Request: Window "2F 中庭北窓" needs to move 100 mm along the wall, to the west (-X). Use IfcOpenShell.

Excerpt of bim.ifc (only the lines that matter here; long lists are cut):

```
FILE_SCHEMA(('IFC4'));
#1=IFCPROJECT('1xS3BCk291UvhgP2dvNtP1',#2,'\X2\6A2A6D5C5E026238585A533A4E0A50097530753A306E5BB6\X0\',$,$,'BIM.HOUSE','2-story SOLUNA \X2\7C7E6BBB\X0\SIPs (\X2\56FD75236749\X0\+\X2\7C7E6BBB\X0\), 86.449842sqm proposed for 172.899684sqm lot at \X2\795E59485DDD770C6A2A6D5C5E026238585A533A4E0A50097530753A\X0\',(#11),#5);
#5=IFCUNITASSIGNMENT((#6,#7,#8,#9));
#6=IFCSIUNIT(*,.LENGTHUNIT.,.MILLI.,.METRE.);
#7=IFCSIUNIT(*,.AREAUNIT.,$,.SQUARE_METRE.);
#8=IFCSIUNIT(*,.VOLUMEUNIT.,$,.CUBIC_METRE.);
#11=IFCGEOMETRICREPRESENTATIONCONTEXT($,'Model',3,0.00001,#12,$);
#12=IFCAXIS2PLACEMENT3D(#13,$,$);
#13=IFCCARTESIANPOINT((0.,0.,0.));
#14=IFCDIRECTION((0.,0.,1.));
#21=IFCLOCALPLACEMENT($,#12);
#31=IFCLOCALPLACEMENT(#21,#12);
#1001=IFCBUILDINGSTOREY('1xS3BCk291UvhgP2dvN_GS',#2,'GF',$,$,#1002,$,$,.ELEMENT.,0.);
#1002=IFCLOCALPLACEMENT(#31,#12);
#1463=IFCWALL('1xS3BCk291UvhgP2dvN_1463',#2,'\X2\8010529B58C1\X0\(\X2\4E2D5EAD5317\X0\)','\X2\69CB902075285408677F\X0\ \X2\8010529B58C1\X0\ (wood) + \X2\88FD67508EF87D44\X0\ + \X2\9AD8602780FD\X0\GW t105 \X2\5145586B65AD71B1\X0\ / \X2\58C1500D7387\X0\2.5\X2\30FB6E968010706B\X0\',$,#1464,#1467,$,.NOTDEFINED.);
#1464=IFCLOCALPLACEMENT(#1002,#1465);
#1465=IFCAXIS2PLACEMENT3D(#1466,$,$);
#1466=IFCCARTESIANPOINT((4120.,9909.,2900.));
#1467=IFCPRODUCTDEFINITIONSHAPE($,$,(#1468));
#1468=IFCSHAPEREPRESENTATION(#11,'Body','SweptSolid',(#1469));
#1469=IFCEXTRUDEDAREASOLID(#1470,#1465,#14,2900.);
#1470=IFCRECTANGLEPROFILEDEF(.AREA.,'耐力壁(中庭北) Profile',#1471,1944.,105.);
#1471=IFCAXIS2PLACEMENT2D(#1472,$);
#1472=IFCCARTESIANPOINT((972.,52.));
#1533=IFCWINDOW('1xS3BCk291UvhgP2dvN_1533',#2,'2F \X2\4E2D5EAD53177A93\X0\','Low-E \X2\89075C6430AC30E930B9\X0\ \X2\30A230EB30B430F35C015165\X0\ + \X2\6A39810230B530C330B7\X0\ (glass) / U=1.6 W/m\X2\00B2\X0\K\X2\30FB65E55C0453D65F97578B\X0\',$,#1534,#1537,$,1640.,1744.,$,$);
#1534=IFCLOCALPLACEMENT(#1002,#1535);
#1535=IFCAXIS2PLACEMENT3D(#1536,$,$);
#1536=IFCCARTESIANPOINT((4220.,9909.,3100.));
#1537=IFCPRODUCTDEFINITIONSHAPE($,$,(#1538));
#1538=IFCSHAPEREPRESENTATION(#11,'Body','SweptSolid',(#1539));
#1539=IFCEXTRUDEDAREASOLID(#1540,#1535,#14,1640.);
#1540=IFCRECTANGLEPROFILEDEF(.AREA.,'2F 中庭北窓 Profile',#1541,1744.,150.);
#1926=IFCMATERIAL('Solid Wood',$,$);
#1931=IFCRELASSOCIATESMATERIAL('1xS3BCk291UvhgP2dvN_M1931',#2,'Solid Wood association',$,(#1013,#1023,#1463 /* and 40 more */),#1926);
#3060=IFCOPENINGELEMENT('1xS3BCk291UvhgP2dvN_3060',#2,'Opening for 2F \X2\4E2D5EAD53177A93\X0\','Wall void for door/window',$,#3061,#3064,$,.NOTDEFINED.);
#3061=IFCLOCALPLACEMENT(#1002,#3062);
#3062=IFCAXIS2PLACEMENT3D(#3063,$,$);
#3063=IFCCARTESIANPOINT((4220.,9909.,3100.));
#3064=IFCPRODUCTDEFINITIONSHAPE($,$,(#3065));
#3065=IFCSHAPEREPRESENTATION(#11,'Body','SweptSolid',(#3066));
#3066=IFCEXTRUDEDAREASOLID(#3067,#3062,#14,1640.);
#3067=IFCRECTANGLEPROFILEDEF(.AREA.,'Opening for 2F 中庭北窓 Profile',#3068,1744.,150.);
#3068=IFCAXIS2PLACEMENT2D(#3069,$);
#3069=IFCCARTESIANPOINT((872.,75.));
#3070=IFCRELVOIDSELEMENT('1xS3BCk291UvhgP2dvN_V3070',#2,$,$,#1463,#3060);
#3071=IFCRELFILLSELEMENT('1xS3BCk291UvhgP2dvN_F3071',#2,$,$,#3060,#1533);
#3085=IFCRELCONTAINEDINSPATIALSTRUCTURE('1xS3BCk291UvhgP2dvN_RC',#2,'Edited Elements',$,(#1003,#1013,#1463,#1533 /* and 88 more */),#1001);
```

```python
import ifcopenshell
import ifcopenshell.api.geometry
import ifcopenshell.util.placement

model = ifcopenshell.open("bim.ifc")

window = model.by_id(1533)
opening = window.FillsVoids[0].RelatingOpeningElement
wall = opening.VoidsElements[0].RelatingBuildingElement

wall_matrix = ifcopenshell.util.placement.get_local_placement(wall.ObjectPlacement)
shift = wall_matrix[:3, 0] * -100.0
before = ifcopenshell.util.placement.get_local_placement(window.ObjectPlacement)[:3, 3].copy()

# The window is not placed relative to its opening, so move both.
for product in (opening, window):
    matrix = ifcopenshell.util.placement.get_local_placement(product.ObjectPlacement)
    matrix[:3, 3] += shift
    ifcopenshell.api.geometry.edit_object_placement(model, product=product, matrix=matrix, is_si=False)

after = ifcopenshell.util.placement.get_local_placement(window.ObjectPlacement)[:3, 3]
print("window moved by", (after - before).round(3) + 0.0)

model.write("bim-out.ifc")
```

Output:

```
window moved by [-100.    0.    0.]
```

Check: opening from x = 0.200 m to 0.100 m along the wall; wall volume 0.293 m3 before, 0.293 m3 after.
